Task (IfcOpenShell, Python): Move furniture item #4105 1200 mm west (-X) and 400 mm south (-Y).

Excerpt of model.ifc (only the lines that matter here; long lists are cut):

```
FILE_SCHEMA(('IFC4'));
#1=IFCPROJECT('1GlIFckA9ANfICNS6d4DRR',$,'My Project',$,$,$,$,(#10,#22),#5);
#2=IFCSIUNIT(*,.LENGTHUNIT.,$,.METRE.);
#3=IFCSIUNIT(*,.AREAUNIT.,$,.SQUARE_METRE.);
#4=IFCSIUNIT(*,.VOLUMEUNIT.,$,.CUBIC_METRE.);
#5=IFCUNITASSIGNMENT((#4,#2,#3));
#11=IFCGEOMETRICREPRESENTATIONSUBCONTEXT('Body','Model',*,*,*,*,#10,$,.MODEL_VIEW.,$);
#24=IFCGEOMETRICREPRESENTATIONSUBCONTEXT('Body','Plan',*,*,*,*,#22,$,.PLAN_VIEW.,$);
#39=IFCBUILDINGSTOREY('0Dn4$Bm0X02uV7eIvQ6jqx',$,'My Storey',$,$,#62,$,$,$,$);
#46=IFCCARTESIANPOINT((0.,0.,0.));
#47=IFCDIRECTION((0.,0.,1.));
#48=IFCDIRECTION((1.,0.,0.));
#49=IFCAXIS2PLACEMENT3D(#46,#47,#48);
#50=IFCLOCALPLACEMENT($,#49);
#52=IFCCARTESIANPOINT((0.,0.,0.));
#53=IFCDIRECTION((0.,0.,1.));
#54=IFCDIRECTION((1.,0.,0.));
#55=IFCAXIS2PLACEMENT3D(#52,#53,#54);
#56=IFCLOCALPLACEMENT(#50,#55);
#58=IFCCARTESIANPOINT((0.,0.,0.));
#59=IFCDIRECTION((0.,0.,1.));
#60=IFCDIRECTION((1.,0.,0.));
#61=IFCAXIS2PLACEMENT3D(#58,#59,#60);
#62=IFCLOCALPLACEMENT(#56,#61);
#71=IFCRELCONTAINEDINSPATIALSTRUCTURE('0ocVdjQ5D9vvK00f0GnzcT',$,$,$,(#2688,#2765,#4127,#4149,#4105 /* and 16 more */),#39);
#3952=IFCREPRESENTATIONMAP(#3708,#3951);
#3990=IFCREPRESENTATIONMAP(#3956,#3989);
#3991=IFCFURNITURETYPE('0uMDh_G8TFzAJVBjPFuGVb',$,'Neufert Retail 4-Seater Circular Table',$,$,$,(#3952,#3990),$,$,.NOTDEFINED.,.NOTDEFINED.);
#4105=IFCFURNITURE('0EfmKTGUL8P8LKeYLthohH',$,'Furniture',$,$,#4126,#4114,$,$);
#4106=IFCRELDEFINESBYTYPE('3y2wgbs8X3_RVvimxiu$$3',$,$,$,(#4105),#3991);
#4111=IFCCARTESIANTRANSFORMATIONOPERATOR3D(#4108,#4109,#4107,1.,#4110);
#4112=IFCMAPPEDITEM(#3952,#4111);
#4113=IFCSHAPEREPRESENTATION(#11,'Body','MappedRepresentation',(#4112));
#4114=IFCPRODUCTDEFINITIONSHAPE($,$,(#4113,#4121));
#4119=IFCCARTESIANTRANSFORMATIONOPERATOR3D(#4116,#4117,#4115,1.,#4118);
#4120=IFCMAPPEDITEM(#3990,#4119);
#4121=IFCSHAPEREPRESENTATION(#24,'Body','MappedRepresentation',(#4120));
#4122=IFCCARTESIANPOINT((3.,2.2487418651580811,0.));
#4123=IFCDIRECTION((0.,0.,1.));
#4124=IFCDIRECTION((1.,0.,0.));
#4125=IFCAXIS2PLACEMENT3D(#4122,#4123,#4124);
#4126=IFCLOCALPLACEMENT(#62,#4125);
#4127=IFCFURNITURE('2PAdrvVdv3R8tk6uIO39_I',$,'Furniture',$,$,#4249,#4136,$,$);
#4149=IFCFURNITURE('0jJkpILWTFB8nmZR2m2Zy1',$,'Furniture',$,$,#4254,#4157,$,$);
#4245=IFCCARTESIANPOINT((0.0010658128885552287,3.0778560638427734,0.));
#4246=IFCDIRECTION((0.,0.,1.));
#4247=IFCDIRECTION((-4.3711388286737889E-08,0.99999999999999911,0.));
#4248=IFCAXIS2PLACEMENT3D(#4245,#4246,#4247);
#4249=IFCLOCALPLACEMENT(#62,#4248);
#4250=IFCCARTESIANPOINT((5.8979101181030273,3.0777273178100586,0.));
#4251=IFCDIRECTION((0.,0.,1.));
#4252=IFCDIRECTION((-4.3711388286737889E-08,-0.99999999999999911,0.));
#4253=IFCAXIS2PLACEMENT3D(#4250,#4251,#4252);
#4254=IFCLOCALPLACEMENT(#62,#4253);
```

```python
import ifcopenshell
import ifcopenshell.api.geometry
import ifcopenshell.util.placement
import ifcopenshell.util.unit

model = ifcopenshell.open("model.ifc")
unit_scale = ifcopenshell.util.unit.calculate_unit_scale(model)

item = model.by_guid("0EfmKTGUL8P8LKeYLthohH")
matrix = ifcopenshell.util.placement.get_local_placement(item.ObjectPlacement)
matrix[0, 3] -= 1.2 / unit_scale
matrix[1, 3] -= 0.4 / unit_scale
ifcopenshell.api.geometry.edit_object_placement(model, product=item, matrix=matrix, is_si=False)

print(ifcopenshell.util.placement.get_local_placement(item.ObjectPlacement).round(3) + 0.0)

model.write("model_rev.ifc")
```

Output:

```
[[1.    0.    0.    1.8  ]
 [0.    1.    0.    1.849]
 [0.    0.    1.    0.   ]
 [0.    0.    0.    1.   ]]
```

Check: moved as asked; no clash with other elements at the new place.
